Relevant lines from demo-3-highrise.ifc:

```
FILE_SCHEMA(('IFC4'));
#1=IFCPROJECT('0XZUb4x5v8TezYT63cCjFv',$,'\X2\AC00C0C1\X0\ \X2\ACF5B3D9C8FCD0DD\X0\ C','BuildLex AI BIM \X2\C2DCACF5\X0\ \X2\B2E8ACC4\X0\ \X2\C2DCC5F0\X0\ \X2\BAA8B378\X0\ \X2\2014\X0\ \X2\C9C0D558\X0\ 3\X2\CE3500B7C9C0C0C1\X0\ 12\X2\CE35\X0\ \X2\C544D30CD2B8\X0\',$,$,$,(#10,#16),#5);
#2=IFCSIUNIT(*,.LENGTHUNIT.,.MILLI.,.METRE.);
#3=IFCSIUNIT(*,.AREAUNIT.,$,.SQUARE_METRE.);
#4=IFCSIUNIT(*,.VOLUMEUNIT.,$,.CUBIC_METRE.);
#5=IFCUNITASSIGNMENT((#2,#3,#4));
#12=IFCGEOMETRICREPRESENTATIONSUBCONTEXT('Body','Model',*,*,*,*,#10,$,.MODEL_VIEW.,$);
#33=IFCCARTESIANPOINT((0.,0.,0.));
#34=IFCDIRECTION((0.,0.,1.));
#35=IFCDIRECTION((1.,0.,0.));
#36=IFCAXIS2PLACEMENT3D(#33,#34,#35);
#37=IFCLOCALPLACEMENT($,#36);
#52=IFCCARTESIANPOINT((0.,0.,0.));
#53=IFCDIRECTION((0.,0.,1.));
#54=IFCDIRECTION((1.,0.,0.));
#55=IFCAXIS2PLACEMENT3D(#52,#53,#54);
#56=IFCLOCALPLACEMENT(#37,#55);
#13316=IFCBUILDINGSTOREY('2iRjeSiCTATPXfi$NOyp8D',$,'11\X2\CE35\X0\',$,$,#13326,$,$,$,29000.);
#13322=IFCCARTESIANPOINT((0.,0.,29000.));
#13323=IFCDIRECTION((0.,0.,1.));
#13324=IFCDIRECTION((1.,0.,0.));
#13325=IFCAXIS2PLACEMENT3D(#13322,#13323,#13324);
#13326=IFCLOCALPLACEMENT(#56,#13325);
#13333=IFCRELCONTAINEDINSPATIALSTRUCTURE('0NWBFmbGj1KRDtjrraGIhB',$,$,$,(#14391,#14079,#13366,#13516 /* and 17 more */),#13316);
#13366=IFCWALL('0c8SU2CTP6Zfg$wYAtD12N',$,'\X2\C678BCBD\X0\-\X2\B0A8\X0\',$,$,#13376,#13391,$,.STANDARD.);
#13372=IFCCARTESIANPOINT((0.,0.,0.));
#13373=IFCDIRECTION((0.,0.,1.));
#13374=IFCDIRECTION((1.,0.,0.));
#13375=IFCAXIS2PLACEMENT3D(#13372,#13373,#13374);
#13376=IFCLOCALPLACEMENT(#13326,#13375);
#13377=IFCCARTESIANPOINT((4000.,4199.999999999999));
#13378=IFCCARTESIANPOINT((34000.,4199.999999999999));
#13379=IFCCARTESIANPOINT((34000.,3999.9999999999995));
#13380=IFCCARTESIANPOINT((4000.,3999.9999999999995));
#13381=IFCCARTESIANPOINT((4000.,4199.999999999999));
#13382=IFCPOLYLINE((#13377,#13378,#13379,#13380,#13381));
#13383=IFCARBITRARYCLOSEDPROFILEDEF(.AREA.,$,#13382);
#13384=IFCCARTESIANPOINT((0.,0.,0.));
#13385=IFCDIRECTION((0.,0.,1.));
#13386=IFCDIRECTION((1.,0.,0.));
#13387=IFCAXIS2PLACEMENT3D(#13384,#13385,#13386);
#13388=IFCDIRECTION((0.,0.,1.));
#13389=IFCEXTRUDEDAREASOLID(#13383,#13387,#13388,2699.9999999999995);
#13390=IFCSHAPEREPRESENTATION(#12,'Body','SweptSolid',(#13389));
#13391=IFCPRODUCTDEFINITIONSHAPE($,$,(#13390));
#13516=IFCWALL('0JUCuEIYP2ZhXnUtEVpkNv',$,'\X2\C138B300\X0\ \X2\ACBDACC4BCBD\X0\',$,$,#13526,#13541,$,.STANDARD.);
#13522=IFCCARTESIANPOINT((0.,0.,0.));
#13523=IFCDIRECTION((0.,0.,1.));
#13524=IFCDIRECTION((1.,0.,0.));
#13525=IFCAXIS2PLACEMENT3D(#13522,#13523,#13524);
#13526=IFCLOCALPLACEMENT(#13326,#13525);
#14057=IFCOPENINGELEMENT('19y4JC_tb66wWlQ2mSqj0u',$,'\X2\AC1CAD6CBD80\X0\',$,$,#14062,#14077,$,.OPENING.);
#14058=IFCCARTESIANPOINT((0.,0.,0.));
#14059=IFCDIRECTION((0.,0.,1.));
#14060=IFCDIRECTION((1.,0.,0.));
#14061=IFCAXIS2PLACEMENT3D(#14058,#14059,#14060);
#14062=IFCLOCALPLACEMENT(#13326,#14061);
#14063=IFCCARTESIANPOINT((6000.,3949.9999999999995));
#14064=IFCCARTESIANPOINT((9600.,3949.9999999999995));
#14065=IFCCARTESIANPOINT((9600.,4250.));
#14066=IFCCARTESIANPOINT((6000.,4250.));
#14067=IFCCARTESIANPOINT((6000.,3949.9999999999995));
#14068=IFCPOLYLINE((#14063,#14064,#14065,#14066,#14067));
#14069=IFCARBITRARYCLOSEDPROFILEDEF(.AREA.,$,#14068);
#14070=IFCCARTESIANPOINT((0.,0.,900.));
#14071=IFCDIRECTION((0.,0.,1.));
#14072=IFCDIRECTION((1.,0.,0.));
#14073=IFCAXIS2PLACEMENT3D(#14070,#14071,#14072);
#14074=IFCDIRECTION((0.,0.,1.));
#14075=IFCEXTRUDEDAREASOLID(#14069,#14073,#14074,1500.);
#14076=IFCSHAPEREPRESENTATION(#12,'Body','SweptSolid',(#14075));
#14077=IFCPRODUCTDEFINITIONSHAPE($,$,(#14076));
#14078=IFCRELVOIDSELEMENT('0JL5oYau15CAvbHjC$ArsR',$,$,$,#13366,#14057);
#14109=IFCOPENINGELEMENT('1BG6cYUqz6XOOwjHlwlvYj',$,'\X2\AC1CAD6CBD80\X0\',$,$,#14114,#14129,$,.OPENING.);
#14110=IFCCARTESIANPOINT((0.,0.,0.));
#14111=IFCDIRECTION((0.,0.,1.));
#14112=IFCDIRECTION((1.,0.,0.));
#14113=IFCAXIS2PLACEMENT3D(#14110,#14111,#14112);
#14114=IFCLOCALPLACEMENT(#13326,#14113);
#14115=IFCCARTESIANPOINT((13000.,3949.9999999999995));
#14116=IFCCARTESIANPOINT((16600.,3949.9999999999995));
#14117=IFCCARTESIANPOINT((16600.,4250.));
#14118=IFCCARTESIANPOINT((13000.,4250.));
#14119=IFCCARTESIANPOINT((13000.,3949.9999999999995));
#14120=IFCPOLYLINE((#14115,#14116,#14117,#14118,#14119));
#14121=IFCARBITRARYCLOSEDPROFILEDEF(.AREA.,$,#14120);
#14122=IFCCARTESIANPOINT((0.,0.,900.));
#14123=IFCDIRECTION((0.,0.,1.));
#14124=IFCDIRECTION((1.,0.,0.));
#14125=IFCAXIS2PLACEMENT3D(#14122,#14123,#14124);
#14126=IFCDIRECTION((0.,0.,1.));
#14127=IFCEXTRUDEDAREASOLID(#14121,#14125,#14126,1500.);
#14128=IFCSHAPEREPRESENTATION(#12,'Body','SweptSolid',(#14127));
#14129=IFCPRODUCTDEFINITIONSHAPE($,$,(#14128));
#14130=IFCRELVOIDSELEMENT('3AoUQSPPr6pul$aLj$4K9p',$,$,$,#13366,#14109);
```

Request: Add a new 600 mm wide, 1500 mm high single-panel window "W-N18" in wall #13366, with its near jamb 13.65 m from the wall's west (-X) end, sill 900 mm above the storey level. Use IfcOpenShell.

```python
import numpy as np
import ifcopenshell
import ifcopenshell.api.feature
import ifcopenshell.api.geometry
import ifcopenshell.api.root
import ifcopenshell.api.spatial
import ifcopenshell.geom
import ifcopenshell.util.element
import ifcopenshell.util.placement
import ifcopenshell.util.representation
import ifcopenshell.util.shape
import ifcopenshell.util.unit

model = ifcopenshell.open("demo-3-highrise.ifc")
unit_scale = ifcopenshell.util.unit.calculate_unit_scale(model)
settings = ifcopenshell.geom.settings()


def volume(element):
    """Net volume in cubic metres, openings subtracted."""
    shape = ifcopenshell.geom.create_shape(settings, element)
    return ifcopenshell.util.shape.get_volume(shape.geometry)


wall = model.by_guid("0c8SU2CTP6Zfg$wYAtD12N")
storey = ifcopenshell.util.element.get_container(wall, ifc_class="IfcBuildingStorey")
context = ifcopenshell.util.representation.get_context(model, "Model", "Body", "MODEL_VIEW")
before = volume(wall)

width, height, from_end, sill = 0.6, 1.5, 13.65, 0.9  # metres

# The wall runs along its own X axis, and the end named is its -X end.
wall_shape = ifcopenshell.geom.create_shape(settings, wall)
x, y, z = ifcopenshell.util.shape.get_vertices(wall_shape.geometry).T
start = x.min() + from_end
face, thickness = float(y.min()), float(y.max() - y.min())
wall_matrix = ifcopenshell.util.placement.get_local_placement(wall.ObjectPlacement)
level = ifcopenshell.util.placement.get_local_placement(storey.ObjectPlacement)[2, 3]


def in_wall(x, y):
    """Placement at x, y metres in the wall's axes, at sill height."""
    matrix = wall_matrix.copy()
    matrix[:, 3] = wall_matrix @ np.array([x / unit_scale, y / unit_scale, 0.0, 1.0])
    matrix[2, 3] = level + sill / unit_scale
    return matrix


# Opening: a box that overshoots both wall faces by 50 mm.
opening = ifcopenshell.api.root.create_entity(model, ifc_class="IfcOpeningElement", predefined_type="OPENING")
box = ifcopenshell.api.geometry.add_wall_representation(
    model, context=context, length=width, height=height, thickness=thickness + 0.1
)
ifcopenshell.api.geometry.assign_representation(model, product=opening, representation=box)
ifcopenshell.api.geometry.edit_object_placement(model, product=opening, matrix=in_wall(start, face - 0.05), is_si=False)
ifcopenshell.api.feature.add_feature(model, feature=opening, element=wall)

window = ifcopenshell.api.root.create_entity(model, ifc_class="IfcWindow", name="W-N18", predefined_type="WINDOW")
window.OverallWidth, window.OverallHeight = width / unit_scale, height / unit_scale
window.PartitioningType = "SINGLE_PANEL"
body = ifcopenshell.api.geometry.add_window_representation(
    model,
    context=context,
    overall_width=window.OverallWidth,
    overall_height=window.OverallHeight,
    partition_type="SINGLE_PANEL",
)
ifcopenshell.api.geometry.assign_representation(model, product=window, representation=body)
ifcopenshell.api.spatial.assign_container(model, products=[window], relating_structure=storey)
ifcopenshell.api.feature.add_filling(model, opening=opening, element=window)

# Centre the window in the wall's thickness.
ifcopenshell.api.geometry.edit_object_placement(model, product=window, matrix=in_wall(start, face), is_si=False)
window_shape = ifcopenshell.geom.create_shape(settings, window)
depth = ifcopenshell.util.shape.get_vertices(window_shape.geometry)[:, 1]
offset = face + thickness / 2 - (depth.min() + depth.max()) / 2
ifcopenshell.api.geometry.edit_object_placement(model, product=window, matrix=in_wall(start, offset), is_si=False)

after = volume(wall)

print(f"wall volume {before:.3f} -> {after:.3f} m3")

model.write("demo-3-highrise_rev.ifc")
```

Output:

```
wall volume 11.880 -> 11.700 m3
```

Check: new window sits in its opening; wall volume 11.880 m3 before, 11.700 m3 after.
